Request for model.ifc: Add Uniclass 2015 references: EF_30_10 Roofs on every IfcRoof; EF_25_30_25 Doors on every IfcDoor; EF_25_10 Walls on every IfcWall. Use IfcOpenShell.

First a look at what the model holds.

```python
import ifcopenshell

model = ifcopenshell.open("model.ifc")
print(model.schema)
print("classifications:", [c.Name for c in model.by_type("IfcClassification")])
for ifc_class in ("IfcDoor", "IfcRoof", "IfcStair", "IfcWall", "IfcWindow"):
    print(ifc_class, len(model.by_type(ifc_class)))
```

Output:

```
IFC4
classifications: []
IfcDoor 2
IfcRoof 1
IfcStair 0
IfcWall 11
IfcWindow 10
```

```python
import ifcopenshell
import ifcopenshell.api.classification

model = ifcopenshell.open("model.ifc")

system = ifcopenshell.api.classification.add_classification(model, classification="Uniclass 2015")

codes = {
    "IfcRoof": ("EF_30_10", "Roofs"),
    "IfcDoor": ("EF_25_30_25", "Doors"),
    "IfcWall": ("EF_25_10", "Walls"),
}
for ifc_class, (code, name) in codes.items():
    products = model.by_type(ifc_class)
    ifcopenshell.api.classification.add_reference(
        model, products=products, classification=system, identification=code, name=name
    )
    print(code, len(products))

model.write("model_edited.ifc")
```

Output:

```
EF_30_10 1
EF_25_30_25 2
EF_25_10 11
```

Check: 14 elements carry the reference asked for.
